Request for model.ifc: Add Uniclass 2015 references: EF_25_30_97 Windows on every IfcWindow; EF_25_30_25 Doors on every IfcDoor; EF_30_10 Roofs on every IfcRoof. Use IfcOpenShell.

First a look at what the model holds.

```python
import ifcopenshell

model = ifcopenshell.open("model.ifc")
print(model.schema)
print("classifications:", [c.Name for c in model.by_type("IfcClassification")])
for ifc_class in ("IfcDoor", "IfcRoof", "IfcStair", "IfcWall", "IfcWindow"):
    print(ifc_class, len(model.by_type(ifc_class)))
```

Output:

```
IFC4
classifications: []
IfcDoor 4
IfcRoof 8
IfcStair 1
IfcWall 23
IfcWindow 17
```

```python
import ifcopenshell
import ifcopenshell.api.classification

model = ifcopenshell.open("model.ifc")

system = ifcopenshell.api.classification.add_classification(model, classification="Uniclass 2015")

codes = {
    "IfcWindow": ("EF_25_30_97", "Windows"),
    "IfcDoor": ("EF_25_30_25", "Doors"),
    "IfcRoof": ("EF_30_10", "Roofs"),
}
for ifc_class, (code, name) in codes.items():
    products = model.by_type(ifc_class)
    ifcopenshell.api.classification.add_reference(
        model, products=products, classification=system, identification=code, name=name
    )
    print(code, len(products))

model.write("model_v2.ifc")
```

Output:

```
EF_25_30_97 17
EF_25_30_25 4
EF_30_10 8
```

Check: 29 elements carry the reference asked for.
